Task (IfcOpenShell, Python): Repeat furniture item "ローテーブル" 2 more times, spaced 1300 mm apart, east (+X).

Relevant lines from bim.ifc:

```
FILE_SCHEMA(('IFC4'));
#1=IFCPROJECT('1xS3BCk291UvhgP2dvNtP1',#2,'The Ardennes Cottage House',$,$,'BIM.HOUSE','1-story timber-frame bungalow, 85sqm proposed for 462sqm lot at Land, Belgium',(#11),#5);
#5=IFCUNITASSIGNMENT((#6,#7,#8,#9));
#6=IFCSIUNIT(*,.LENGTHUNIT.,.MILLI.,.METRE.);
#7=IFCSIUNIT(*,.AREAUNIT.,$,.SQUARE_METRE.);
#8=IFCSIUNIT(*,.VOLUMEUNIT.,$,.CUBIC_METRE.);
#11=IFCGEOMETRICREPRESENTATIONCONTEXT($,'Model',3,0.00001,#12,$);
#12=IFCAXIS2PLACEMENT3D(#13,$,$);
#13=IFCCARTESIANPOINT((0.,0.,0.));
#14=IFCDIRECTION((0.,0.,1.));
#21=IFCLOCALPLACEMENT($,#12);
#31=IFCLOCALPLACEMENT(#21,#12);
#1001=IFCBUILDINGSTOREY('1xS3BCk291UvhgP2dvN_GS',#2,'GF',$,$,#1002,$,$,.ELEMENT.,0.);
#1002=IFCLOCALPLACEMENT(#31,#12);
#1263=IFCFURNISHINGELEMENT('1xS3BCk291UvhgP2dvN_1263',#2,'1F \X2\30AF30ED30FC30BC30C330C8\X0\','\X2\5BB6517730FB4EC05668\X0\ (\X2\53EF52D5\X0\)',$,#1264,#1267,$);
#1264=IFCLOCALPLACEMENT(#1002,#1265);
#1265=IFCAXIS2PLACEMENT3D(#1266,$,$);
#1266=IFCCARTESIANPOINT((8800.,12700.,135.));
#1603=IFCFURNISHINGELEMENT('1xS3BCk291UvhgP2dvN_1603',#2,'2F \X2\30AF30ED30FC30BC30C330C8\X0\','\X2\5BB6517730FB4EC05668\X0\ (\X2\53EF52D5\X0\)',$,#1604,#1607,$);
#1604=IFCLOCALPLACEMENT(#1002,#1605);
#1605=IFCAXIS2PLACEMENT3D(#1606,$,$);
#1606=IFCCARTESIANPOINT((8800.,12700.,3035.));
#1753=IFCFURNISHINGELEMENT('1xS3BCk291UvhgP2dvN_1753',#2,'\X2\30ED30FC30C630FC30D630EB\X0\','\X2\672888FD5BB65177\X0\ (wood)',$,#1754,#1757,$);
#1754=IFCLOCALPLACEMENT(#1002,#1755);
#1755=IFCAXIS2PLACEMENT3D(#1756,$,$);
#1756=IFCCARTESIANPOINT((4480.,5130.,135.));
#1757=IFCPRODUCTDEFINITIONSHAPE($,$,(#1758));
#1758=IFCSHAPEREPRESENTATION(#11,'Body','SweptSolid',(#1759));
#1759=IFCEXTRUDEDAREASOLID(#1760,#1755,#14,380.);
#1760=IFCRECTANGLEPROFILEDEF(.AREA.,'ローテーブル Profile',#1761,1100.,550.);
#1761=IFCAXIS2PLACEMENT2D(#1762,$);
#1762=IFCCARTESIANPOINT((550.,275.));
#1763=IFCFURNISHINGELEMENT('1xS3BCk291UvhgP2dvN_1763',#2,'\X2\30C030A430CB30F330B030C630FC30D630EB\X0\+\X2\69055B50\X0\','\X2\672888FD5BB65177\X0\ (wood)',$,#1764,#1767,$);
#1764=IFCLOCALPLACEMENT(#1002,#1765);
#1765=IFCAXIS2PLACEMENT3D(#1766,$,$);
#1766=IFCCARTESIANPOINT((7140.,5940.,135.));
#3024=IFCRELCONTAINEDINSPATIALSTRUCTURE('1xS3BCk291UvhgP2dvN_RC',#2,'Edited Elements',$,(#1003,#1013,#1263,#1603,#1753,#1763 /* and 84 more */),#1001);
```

```python
import numpy as np
import ifcopenshell
import ifcopenshell.api.geometry
import ifcopenshell.api.root
import ifcopenshell.util.element
import ifcopenshell.util.placement

model = ifcopenshell.open("bim.ifc")


def reuse_history(source, copy):
    """copy_class also copies each property set's owner history, people and application; keep the originals."""
    for rel in copy.IsDefinedBy:
        if rel.is_a("IfcRelDefinesByProperties") and (history := rel.RelatingPropertyDefinition.OwnerHistory):
            rel.RelatingPropertyDefinition.OwnerHistory = source.OwnerHistory
            ifcopenshell.util.element.remove_deep2(model, history)


source = model.by_guid("1xS3BCk291UvhgP2dvN_1753")
base = ifcopenshell.util.placement.get_local_placement(source.ObjectPlacement)
step = np.array([1.0, 0.0, 0.0]) * 1300.0

for i in range(1, 3):
    copy = ifcopenshell.api.root.copy_class(model, product=source)
    copy.Representation = ifcopenshell.util.element.copy_deep(
        model, source.Representation, exclude=["IfcGeometricRepresentationContext", "IfcRepresentationMap"]
    )
    reuse_history(source, copy)
    matrix = base.copy()
    matrix[:3, 3] += i * step
    print("added at", matrix[:3, 3].round(3) + 0.0)
    ifcopenshell.api.geometry.edit_object_placement(model, product=copy, matrix=matrix, is_si=False)

model.write("bim_rev.ifc")
```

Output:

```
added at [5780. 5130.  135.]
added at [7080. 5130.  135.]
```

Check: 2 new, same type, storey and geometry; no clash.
